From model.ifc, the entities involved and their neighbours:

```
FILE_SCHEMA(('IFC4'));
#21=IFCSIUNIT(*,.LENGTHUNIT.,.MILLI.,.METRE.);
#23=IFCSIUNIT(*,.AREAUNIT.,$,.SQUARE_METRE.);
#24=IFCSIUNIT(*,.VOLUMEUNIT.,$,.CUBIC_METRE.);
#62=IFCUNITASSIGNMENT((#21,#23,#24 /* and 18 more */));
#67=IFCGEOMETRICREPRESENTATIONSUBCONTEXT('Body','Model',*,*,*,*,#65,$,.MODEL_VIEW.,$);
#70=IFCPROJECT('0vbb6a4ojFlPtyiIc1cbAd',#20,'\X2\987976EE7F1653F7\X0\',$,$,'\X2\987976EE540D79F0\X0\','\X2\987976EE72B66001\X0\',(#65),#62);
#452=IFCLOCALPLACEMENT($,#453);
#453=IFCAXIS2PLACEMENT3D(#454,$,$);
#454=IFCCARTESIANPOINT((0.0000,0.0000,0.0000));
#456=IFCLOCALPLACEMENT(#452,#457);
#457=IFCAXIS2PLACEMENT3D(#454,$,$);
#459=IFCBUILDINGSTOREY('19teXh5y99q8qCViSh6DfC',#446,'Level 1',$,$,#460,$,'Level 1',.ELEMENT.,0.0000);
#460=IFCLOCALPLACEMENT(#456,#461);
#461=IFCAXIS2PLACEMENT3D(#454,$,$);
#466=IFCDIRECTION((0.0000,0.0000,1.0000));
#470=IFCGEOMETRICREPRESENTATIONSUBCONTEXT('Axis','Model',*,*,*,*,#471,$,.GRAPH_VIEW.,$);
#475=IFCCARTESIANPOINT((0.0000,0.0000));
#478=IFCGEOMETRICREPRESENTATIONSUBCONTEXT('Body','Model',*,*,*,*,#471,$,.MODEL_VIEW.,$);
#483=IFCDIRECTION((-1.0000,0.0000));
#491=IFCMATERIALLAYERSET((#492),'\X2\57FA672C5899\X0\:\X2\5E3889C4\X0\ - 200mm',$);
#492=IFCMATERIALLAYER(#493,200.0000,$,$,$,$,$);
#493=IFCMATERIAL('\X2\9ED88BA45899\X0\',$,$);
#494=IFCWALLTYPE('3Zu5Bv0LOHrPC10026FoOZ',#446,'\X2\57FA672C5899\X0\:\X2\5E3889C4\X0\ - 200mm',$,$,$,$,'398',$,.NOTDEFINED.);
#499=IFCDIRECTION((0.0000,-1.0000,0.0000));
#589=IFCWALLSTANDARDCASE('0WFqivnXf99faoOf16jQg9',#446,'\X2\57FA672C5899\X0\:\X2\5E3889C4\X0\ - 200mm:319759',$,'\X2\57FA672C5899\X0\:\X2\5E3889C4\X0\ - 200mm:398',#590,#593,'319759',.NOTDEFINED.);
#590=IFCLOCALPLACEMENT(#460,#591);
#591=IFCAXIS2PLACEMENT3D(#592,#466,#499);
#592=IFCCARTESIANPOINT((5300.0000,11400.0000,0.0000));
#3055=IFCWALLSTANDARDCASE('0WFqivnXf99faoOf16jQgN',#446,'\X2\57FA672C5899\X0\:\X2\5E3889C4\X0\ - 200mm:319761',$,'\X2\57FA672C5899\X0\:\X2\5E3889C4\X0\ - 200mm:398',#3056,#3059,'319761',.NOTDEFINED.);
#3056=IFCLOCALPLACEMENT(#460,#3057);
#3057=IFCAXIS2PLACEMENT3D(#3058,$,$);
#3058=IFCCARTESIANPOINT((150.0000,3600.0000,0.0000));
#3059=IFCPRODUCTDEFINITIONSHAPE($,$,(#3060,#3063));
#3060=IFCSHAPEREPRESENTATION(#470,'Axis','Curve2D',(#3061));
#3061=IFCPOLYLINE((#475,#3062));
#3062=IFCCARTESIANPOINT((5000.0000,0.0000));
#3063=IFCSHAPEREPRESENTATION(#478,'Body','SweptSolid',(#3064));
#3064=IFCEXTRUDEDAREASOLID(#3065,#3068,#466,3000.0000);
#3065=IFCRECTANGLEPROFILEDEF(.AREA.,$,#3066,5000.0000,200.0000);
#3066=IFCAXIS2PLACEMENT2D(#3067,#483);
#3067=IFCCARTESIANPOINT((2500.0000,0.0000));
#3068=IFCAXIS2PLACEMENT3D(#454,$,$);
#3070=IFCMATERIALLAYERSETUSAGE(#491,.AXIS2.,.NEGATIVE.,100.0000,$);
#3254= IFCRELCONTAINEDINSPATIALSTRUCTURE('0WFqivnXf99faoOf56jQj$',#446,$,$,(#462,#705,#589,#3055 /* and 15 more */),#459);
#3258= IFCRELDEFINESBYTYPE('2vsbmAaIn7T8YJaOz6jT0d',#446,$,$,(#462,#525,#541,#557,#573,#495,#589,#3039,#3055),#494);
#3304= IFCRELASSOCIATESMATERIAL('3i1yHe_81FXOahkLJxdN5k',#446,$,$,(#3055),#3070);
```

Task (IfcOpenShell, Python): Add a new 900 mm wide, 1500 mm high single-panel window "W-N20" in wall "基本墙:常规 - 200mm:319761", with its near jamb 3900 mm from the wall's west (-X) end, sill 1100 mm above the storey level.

```python
import numpy as np
import ifcopenshell
import ifcopenshell.api.feature
import ifcopenshell.api.geometry
import ifcopenshell.api.root
import ifcopenshell.api.spatial
import ifcopenshell.geom
import ifcopenshell.util.element
import ifcopenshell.util.placement
import ifcopenshell.util.representation
import ifcopenshell.util.shape
import ifcopenshell.util.unit

model = ifcopenshell.open("model.ifc")
unit_scale = ifcopenshell.util.unit.calculate_unit_scale(model)
settings = ifcopenshell.geom.settings()


def volume(element):
    """Net volume in cubic metres, openings subtracted."""
    shape = ifcopenshell.geom.create_shape(settings, element)
    return ifcopenshell.util.shape.get_volume(shape.geometry)


wall = model.by_guid("0WFqivnXf99faoOf16jQgN")
storey = ifcopenshell.util.element.get_container(wall, ifc_class="IfcBuildingStorey")
context = ifcopenshell.util.representation.get_context(model, "Model", "Body", "MODEL_VIEW")
before = volume(wall)

width, height, from_end, sill = 0.9, 1.5, 3.9, 1.1  # metres

# The wall runs along its own X axis, and the end named is its -X end.
wall_shape = ifcopenshell.geom.create_shape(settings, wall)
x, y, z = ifcopenshell.util.shape.get_vertices(wall_shape.geometry).T
start = x.min() + from_end
face, thickness = float(y.min()), float(y.max() - y.min())
wall_matrix = ifcopenshell.util.placement.get_local_placement(wall.ObjectPlacement)
level = ifcopenshell.util.placement.get_local_placement(storey.ObjectPlacement)[2, 3]


def in_wall(x, y):
    """Placement at x, y metres in the wall's axes, at sill height."""
    matrix = wall_matrix.copy()
    matrix[:, 3] = wall_matrix @ np.array([x / unit_scale, y / unit_scale, 0.0, 1.0])
    matrix[2, 3] = level + sill / unit_scale
    return matrix


# Opening: a box that overshoots both wall faces by 50 mm.
opening = ifcopenshell.api.root.create_entity(model, ifc_class="IfcOpeningElement", predefined_type="OPENING")
box = ifcopenshell.api.geometry.add_wall_representation(
    model, context=context, length=width, height=height, thickness=thickness + 0.1
)
ifcopenshell.api.geometry.assign_representation(model, product=opening, representation=box)
ifcopenshell.api.geometry.edit_object_placement(model, product=opening, matrix=in_wall(start, face - 0.05), is_si=False)
ifcopenshell.api.feature.add_feature(model, feature=opening, element=wall)

window = ifcopenshell.api.root.create_entity(model, ifc_class="IfcWindow", name="W-N20", predefined_type="WINDOW")
window.OverallWidth, window.OverallHeight = width / unit_scale, height / unit_scale
window.PartitioningType = "SINGLE_PANEL"
body = ifcopenshell.api.geometry.add_window_representation(
    model,
    context=context,
    overall_width=window.OverallWidth,
    overall_height=window.OverallHeight,
    partition_type="SINGLE_PANEL",
)
ifcopenshell.api.geometry.assign_representation(model, product=window, representation=body)
ifcopenshell.api.spatial.assign_container(model, products=[window], relating_structure=storey)
ifcopenshell.api.feature.add_filling(model, opening=opening, element=window)

# Centre the window in the wall's thickness.
ifcopenshell.api.geometry.edit_object_placement(model, product=window, matrix=in_wall(start, face), is_si=False)
window_shape = ifcopenshell.geom.create_shape(settings, window)
depth = ifcopenshell.util.shape.get_vertices(window_shape.geometry)[:, 1]
offset = face + thickness / 2 - (depth.min() + depth.max()) / 2
ifcopenshell.api.geometry.edit_object_placement(model, product=window, matrix=in_wall(start, offset), is_si=False)

after = volume(wall)

print(f"wall volume {before:.3f} -> {after:.3f} m3")

model.write("model_updated.ifc")
```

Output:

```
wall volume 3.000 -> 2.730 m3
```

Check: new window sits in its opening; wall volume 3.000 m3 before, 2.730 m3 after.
